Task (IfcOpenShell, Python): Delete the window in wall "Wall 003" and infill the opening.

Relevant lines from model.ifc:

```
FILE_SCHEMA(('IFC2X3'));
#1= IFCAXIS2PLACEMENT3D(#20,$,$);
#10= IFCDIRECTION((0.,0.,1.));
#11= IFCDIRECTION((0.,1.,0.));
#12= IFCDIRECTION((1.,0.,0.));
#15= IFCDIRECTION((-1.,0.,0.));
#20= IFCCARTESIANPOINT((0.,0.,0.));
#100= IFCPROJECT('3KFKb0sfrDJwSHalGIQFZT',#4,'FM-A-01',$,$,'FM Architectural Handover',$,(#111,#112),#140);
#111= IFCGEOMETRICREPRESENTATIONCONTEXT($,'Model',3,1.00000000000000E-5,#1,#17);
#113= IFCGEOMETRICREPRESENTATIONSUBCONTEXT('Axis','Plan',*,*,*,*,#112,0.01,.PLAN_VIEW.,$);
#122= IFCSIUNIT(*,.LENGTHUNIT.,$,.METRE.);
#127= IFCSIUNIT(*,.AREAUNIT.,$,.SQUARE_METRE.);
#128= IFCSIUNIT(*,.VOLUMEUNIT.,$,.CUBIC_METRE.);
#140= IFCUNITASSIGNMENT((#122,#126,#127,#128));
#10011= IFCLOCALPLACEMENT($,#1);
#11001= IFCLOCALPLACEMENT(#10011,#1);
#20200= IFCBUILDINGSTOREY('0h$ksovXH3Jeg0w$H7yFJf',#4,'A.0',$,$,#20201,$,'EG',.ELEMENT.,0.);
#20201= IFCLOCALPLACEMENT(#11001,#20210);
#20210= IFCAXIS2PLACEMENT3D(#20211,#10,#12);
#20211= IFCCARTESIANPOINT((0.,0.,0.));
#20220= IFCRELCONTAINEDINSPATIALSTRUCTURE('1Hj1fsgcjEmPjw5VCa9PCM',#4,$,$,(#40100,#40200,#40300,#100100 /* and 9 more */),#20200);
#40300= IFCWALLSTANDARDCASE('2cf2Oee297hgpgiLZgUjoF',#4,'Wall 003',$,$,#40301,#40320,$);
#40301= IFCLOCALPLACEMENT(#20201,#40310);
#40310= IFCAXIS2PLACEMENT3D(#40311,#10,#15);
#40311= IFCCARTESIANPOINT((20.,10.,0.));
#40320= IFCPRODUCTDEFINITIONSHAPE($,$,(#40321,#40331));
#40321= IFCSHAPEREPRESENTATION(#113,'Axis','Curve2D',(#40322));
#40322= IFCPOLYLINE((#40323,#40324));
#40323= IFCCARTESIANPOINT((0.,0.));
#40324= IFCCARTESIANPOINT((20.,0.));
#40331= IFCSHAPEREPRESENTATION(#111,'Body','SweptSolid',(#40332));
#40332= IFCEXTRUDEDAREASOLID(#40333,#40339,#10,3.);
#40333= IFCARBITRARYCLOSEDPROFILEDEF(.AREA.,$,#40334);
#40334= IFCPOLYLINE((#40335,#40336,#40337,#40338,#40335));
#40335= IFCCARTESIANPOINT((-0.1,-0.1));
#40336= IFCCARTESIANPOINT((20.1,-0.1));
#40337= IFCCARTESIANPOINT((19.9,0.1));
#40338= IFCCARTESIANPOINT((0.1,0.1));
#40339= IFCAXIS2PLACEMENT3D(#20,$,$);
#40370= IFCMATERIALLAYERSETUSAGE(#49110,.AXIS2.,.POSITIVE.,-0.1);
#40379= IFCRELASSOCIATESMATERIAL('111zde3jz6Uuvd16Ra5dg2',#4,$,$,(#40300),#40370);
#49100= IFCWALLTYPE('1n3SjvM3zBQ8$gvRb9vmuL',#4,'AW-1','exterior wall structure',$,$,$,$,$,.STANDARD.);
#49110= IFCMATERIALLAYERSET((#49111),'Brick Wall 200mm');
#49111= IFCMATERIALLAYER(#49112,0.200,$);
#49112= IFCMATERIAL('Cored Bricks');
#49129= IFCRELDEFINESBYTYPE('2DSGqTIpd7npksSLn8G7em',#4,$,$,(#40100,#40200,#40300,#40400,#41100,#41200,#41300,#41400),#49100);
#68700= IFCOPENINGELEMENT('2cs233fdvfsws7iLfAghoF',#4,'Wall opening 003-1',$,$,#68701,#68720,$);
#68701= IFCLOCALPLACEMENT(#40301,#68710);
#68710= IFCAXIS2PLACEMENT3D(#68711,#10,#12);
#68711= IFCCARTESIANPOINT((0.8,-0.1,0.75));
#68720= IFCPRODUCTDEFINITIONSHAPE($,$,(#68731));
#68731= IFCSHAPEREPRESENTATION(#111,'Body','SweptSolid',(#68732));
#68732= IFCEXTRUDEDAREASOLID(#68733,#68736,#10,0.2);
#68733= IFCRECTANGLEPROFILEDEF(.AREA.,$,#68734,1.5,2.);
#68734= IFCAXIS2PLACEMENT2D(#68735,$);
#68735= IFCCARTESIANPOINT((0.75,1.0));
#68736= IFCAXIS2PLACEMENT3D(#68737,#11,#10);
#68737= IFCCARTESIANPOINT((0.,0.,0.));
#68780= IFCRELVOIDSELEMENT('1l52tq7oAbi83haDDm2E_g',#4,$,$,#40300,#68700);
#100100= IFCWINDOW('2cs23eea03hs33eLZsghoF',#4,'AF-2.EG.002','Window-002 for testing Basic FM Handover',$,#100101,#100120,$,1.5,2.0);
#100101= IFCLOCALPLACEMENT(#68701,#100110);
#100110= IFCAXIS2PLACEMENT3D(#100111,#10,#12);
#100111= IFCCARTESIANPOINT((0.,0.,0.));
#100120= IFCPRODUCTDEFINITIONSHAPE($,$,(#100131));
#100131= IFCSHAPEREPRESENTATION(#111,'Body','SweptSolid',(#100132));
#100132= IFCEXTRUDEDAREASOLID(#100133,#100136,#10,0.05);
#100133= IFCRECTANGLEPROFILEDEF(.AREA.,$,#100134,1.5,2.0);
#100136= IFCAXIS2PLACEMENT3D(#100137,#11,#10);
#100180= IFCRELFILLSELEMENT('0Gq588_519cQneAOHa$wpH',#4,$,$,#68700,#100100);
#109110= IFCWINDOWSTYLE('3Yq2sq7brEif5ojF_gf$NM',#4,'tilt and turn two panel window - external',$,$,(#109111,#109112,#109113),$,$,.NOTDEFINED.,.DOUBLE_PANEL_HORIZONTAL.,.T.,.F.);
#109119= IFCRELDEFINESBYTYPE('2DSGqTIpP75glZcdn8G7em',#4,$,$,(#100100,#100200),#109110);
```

```python
import ifcopenshell
import ifcopenshell.api.feature
import ifcopenshell.api.root
import ifcopenshell.geom
import ifcopenshell.util.shape

model = ifcopenshell.open("model.ifc")
settings = ifcopenshell.geom.settings()


def volume(element):
    """Net volume in cubic metres, openings subtracted."""
    shape = ifcopenshell.geom.create_shape(settings, element)
    return ifcopenshell.util.shape.get_volume(shape.geometry)


window = model.by_guid("2cs23eea03hs33eLZsghoF")
opening = window.FillsVoids[0].RelatingOpeningElement
wall = opening.VoidsElements[0].RelatingBuildingElement
before = volume(wall)

ifcopenshell.api.root.remove_product(model, product=window)
ifcopenshell.api.feature.remove_feature(model, feature=opening)

after = volume(wall)

print(f"wall volume {before:.3f} -> {after:.3f} m3")

model.write("model-out.ifc")
```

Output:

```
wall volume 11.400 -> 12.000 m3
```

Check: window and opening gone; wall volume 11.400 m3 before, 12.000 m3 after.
